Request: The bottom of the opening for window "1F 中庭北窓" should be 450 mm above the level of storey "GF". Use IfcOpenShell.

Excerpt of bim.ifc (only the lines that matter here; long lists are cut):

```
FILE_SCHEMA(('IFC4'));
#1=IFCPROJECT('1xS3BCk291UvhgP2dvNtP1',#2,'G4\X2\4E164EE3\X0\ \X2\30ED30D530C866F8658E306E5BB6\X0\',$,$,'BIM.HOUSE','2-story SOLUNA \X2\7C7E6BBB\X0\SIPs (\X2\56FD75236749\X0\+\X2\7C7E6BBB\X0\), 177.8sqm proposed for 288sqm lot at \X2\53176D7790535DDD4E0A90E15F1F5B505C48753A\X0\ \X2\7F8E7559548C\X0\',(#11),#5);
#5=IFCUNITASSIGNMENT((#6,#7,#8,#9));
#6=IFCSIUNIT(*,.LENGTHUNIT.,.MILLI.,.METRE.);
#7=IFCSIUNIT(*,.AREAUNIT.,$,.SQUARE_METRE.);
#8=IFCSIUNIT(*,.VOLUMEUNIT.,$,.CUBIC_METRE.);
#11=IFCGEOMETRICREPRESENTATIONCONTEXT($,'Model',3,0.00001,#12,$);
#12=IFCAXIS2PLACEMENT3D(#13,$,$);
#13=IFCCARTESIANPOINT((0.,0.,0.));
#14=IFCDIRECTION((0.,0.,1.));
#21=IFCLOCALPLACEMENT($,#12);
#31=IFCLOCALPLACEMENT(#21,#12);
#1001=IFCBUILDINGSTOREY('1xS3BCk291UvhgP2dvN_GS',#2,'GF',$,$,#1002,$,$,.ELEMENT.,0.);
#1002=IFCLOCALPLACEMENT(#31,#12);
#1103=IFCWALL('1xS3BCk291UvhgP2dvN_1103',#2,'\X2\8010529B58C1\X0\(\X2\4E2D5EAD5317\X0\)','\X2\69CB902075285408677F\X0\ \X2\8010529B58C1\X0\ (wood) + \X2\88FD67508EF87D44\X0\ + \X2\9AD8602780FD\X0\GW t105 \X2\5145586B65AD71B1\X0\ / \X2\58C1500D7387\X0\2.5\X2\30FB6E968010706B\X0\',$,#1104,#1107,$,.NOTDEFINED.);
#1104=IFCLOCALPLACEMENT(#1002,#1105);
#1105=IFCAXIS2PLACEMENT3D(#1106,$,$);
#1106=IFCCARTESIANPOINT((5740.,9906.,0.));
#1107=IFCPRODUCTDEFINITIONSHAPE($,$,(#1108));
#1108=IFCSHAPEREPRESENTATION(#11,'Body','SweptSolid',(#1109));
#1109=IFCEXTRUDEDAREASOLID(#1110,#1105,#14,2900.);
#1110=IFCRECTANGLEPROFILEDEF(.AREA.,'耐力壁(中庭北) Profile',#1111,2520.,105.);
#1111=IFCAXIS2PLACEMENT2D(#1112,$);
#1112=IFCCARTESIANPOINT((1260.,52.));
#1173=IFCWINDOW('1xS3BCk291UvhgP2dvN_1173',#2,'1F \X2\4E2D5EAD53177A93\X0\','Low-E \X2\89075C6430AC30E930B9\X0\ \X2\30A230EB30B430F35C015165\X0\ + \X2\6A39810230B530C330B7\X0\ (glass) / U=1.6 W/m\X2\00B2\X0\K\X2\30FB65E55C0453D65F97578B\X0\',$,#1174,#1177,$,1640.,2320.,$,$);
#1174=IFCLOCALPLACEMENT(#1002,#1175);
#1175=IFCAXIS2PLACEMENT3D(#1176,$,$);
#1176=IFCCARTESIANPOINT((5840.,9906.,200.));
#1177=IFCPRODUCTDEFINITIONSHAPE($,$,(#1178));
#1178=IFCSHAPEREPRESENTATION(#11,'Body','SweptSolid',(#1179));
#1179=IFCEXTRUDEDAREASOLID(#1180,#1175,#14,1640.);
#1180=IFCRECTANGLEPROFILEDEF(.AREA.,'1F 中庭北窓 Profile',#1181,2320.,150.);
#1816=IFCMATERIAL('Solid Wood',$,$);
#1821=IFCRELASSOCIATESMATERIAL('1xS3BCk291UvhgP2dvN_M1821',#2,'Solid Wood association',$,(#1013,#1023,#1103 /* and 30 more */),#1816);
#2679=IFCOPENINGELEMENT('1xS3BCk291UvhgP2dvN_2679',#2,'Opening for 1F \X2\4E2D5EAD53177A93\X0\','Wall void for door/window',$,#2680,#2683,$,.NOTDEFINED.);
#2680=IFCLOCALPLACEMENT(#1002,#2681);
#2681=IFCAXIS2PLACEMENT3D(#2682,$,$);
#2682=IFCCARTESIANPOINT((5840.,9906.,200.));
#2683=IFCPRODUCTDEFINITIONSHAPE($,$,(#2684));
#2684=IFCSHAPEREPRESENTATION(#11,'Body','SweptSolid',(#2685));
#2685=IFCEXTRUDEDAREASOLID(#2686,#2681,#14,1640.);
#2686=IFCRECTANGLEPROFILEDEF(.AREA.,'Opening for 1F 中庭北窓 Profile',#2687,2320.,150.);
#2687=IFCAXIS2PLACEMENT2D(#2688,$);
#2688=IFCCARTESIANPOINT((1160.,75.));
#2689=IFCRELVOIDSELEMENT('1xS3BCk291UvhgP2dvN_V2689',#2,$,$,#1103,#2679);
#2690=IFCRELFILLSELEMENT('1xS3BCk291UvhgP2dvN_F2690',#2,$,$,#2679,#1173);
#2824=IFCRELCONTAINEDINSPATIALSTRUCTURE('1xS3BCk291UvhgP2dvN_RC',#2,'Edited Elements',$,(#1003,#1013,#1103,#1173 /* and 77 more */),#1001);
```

```python
import numpy as np
import ifcopenshell
import ifcopenshell.api.geometry
import ifcopenshell.geom
import ifcopenshell.util.element
import ifcopenshell.util.placement
import ifcopenshell.util.shape
import ifcopenshell.util.unit

model = ifcopenshell.open("bim.ifc")
unit_scale = ifcopenshell.util.unit.calculate_unit_scale(model)

window = model.by_guid("1xS3BCk291UvhgP2dvN_1173")
opening = window.FillsVoids[0].RelatingOpeningElement
storey = ifcopenshell.util.element.get_container(window, ifc_class="IfcBuildingStorey")
level = ifcopenshell.util.placement.get_local_placement(storey.ObjectPlacement)[2, 3]

# The opening's origin need not be at the sill, so measure its lowest point.
shape = ifcopenshell.geom.create_shape(ifcopenshell.geom.settings(), opening)
bottom = ifcopenshell.util.shape.get_shape_bottom_elevation(shape, shape.geometry) / unit_scale
dz = level + 0.45 / unit_scale - bottom

shift = np.array([0.0, 0.0, dz])
# The window is not placed relative to its opening, so move both.
for product in (opening, window):
    matrix = ifcopenshell.util.placement.get_local_placement(product.ObjectPlacement)
    matrix[:3, 3] += shift
    ifcopenshell.api.geometry.edit_object_placement(model, product=product, matrix=matrix, is_si=False)

print(f"moved by {dz * unit_scale:+.3f} m")

model.write("bim_v2.ifc")
```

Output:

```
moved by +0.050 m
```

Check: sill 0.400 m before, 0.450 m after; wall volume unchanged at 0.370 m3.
